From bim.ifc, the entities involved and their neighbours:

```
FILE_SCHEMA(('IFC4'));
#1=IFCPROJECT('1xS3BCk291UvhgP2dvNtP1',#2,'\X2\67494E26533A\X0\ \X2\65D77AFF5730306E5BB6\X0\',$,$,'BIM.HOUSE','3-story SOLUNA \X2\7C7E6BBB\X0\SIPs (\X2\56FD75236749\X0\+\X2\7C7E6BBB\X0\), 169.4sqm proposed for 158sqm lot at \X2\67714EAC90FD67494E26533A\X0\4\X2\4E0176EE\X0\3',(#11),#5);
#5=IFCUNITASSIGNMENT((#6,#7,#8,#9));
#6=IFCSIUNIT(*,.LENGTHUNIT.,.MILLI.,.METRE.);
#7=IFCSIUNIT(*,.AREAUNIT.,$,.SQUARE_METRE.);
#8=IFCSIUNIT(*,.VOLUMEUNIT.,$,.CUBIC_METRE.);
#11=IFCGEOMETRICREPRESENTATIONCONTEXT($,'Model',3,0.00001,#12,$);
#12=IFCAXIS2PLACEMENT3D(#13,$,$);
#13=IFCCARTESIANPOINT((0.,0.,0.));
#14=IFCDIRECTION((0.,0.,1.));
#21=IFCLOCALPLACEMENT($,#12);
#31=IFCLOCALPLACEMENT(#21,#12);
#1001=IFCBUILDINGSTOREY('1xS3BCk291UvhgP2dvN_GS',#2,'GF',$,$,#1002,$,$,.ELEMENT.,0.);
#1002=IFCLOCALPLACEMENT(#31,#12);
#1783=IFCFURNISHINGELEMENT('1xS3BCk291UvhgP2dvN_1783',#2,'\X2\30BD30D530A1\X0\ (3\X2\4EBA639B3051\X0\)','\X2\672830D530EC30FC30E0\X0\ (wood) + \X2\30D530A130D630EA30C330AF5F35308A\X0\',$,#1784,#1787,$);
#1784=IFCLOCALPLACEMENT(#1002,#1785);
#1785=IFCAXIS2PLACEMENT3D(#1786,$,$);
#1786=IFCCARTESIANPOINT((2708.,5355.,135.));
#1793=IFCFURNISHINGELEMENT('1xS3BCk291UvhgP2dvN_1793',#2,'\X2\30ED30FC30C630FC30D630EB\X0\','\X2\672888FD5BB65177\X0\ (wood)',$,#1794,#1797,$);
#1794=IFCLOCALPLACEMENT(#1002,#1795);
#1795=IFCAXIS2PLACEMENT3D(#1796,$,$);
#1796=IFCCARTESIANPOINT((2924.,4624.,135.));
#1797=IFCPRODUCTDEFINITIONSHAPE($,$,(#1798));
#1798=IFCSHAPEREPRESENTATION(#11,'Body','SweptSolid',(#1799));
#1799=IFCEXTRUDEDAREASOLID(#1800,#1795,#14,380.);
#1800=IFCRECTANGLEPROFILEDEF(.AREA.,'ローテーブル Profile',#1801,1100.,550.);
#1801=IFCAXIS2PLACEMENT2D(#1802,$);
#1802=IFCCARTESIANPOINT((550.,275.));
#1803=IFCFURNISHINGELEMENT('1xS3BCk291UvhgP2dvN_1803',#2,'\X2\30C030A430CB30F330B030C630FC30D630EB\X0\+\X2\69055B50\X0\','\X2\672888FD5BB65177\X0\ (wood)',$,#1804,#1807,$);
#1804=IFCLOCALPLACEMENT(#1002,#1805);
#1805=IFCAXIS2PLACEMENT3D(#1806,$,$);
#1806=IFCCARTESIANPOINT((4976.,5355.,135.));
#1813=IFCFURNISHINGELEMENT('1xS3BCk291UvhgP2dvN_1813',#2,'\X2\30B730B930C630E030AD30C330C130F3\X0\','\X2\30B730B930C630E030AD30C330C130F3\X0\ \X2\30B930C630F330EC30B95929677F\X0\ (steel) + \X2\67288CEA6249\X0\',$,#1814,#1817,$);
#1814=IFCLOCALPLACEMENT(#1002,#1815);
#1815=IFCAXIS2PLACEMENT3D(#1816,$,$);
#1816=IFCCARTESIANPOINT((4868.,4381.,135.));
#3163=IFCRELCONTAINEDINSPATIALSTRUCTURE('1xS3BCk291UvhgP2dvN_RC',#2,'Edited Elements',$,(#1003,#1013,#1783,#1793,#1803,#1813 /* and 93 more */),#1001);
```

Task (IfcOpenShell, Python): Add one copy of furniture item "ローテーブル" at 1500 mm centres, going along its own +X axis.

```python
import ifcopenshell
import ifcopenshell.api.geometry
import ifcopenshell.api.root
import ifcopenshell.util.element
import ifcopenshell.util.placement

model = ifcopenshell.open("bim.ifc")


def reuse_history(source, copy):
    """copy_class also copies each property set's owner history, people and application; keep the originals."""
    for rel in copy.IsDefinedBy:
        if rel.is_a("IfcRelDefinesByProperties") and (history := rel.RelatingPropertyDefinition.OwnerHistory):
            rel.RelatingPropertyDefinition.OwnerHistory = source.OwnerHistory
            ifcopenshell.util.element.remove_deep2(model, history)


source = model.by_id(1793)
base = ifcopenshell.util.placement.get_local_placement(source.ObjectPlacement)
step = base[:3, 0] * 1500.0

for i in range(1, 2):
    copy = ifcopenshell.api.root.copy_class(model, product=source)
    copy.Representation = ifcopenshell.util.element.copy_deep(
        model, source.Representation, exclude=["IfcGeometricRepresentationContext", "IfcRepresentationMap"]
    )
    reuse_history(source, copy)
    matrix = base.copy()
    matrix[:3, 3] += i * step
    print("added at", matrix[:3, 3].round(3) + 0.0)
    ifcopenshell.api.geometry.edit_object_placement(model, product=copy, matrix=matrix, is_si=False)

model.write("bim_updated.ifc")
```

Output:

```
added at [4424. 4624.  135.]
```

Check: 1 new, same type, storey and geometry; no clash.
